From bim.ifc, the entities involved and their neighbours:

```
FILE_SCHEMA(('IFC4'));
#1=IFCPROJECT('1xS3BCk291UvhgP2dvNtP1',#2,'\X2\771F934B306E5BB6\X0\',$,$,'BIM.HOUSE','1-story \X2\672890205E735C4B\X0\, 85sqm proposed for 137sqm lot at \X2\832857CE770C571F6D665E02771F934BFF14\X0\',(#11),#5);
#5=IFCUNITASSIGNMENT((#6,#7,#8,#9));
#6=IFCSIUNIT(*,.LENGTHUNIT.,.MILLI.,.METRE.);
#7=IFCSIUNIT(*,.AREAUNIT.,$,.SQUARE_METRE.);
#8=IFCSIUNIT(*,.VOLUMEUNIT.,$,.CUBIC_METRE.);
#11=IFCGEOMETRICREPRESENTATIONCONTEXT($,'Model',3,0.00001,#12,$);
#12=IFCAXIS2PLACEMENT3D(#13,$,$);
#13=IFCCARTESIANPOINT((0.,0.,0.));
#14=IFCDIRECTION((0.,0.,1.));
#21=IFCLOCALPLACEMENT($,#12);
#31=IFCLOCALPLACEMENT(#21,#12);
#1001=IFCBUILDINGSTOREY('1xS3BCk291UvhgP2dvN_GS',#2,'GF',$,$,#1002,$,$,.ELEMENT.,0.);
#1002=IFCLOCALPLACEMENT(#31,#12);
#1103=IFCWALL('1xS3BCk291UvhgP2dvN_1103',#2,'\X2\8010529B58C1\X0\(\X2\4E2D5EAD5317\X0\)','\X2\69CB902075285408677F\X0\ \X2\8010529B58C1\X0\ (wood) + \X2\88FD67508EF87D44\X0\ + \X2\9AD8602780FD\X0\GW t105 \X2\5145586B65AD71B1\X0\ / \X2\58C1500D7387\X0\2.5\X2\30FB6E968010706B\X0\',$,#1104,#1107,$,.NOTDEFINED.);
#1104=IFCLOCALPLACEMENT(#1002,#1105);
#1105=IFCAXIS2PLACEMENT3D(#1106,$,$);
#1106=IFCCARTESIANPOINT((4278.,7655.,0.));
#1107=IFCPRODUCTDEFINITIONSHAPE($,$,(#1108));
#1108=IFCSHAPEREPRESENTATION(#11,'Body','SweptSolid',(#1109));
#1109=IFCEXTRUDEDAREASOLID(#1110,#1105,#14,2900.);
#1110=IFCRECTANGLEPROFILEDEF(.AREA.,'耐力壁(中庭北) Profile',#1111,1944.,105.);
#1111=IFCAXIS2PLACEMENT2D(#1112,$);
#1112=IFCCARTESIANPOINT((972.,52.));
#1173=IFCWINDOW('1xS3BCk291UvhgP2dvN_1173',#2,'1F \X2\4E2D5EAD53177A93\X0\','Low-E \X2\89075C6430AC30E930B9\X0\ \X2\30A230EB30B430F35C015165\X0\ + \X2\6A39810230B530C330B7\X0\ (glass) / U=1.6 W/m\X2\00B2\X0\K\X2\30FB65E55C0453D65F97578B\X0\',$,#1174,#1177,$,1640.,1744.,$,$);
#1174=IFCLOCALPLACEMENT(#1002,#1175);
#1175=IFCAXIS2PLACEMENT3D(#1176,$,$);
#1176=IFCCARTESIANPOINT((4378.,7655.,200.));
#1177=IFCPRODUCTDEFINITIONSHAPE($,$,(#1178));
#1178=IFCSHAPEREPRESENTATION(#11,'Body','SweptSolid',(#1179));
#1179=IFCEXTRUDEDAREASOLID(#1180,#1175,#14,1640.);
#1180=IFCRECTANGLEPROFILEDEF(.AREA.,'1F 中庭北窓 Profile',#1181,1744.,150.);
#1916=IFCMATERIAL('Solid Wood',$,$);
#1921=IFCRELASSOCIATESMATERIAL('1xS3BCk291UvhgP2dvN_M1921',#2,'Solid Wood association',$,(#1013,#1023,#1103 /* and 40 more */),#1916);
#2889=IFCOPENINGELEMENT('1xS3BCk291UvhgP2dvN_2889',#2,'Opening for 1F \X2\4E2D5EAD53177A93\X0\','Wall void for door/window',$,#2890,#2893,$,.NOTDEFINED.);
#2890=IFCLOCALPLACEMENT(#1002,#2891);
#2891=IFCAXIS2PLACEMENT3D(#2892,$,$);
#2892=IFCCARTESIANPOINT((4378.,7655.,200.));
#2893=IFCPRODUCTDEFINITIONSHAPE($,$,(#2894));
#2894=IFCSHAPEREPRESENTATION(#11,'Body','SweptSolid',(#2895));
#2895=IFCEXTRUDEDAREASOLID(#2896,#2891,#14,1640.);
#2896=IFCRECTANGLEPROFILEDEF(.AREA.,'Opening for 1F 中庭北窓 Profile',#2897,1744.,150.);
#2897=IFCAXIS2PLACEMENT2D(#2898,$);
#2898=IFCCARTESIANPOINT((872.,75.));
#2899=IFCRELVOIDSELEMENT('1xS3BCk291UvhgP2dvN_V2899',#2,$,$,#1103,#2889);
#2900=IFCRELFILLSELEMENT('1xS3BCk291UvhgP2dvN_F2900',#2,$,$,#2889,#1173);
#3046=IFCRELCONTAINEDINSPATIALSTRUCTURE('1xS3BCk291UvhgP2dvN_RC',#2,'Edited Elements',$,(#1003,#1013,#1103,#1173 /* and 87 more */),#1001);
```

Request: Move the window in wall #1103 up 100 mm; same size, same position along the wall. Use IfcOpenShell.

```python
import numpy as np
import ifcopenshell
import ifcopenshell.api.geometry
import ifcopenshell.util.placement
import ifcopenshell.util.unit

model = ifcopenshell.open("bim.ifc")
unit_scale = ifcopenshell.util.unit.calculate_unit_scale(model)

window = model.by_guid("1xS3BCk291UvhgP2dvN_1173")
opening = window.FillsVoids[0].RelatingOpeningElement
dz = 0.1 / unit_scale

shift = np.array([0.0, 0.0, dz])
# The window is not placed relative to its opening, so move both.
for product in (opening, window):
    matrix = ifcopenshell.util.placement.get_local_placement(product.ObjectPlacement)
    matrix[:3, 3] += shift
    ifcopenshell.api.geometry.edit_object_placement(model, product=product, matrix=matrix, is_si=False)

print(f"moved by {dz * unit_scale:+.3f} m")

model.write("bim_rev.ifc")
```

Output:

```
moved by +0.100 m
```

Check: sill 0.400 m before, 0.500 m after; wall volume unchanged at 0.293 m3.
